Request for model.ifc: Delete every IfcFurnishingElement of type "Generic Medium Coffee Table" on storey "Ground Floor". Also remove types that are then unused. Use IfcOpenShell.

First a look at what the model holds.

```python
import ifcopenshell
import ifcopenshell.util.element

model = ifcopenshell.open("model.ifc")
print(model.schema)
storey = next(s for s in model.by_type("IfcBuildingStorey") if s.Name == "Ground Floor")
furniture = [e for e in ifcopenshell.util.element.get_decomposition(storey) if e.is_a("IfcFurnishingElement")]
seen = {}
for e in furniture:
    element_type = ifcopenshell.util.element.get_type(e)
    name = element_type.Name if element_type not in (None, e) else None
    seen[name] = seen.get(name, 0) + 1
for name, count in sorted(seen.items(), key=str):
    print(count, "x", name)
```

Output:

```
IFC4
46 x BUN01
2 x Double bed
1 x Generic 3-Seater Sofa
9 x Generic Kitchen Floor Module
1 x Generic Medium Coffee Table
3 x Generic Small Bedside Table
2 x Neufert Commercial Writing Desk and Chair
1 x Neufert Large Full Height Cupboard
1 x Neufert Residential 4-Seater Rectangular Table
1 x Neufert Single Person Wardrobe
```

```python
import ifcopenshell
import ifcopenshell.api.root
import ifcopenshell.util.element

model = ifcopenshell.open("model.ifc")

storey = next(s for s in model.by_type("IfcBuildingStorey") if s.Name == "Ground Floor")
furniture = [e for e in ifcopenshell.util.element.get_decomposition(storey) if e.is_a("IfcFurnishingElement")]
targets = [e for e in furniture if (t := ifcopenshell.util.element.get_type(e)) not in (None, e) and t.Name == "Generic Medium Coffee Table"]
types = {ifcopenshell.util.element.get_type(e) for e in targets} - {None, *targets}

for e in targets:
    ifcopenshell.api.root.remove_product(model, product=e)
print(len(targets), "removed")

unused = [t for t in types if not ifcopenshell.util.element.get_types(t)]
for t in unused:
    ifcopenshell.api.root.remove_product(model, product=t)
print(len(unused), "unused types removed")

model.write("model_rev.ifc")
```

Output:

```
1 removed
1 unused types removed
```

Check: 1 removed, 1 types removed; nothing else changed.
